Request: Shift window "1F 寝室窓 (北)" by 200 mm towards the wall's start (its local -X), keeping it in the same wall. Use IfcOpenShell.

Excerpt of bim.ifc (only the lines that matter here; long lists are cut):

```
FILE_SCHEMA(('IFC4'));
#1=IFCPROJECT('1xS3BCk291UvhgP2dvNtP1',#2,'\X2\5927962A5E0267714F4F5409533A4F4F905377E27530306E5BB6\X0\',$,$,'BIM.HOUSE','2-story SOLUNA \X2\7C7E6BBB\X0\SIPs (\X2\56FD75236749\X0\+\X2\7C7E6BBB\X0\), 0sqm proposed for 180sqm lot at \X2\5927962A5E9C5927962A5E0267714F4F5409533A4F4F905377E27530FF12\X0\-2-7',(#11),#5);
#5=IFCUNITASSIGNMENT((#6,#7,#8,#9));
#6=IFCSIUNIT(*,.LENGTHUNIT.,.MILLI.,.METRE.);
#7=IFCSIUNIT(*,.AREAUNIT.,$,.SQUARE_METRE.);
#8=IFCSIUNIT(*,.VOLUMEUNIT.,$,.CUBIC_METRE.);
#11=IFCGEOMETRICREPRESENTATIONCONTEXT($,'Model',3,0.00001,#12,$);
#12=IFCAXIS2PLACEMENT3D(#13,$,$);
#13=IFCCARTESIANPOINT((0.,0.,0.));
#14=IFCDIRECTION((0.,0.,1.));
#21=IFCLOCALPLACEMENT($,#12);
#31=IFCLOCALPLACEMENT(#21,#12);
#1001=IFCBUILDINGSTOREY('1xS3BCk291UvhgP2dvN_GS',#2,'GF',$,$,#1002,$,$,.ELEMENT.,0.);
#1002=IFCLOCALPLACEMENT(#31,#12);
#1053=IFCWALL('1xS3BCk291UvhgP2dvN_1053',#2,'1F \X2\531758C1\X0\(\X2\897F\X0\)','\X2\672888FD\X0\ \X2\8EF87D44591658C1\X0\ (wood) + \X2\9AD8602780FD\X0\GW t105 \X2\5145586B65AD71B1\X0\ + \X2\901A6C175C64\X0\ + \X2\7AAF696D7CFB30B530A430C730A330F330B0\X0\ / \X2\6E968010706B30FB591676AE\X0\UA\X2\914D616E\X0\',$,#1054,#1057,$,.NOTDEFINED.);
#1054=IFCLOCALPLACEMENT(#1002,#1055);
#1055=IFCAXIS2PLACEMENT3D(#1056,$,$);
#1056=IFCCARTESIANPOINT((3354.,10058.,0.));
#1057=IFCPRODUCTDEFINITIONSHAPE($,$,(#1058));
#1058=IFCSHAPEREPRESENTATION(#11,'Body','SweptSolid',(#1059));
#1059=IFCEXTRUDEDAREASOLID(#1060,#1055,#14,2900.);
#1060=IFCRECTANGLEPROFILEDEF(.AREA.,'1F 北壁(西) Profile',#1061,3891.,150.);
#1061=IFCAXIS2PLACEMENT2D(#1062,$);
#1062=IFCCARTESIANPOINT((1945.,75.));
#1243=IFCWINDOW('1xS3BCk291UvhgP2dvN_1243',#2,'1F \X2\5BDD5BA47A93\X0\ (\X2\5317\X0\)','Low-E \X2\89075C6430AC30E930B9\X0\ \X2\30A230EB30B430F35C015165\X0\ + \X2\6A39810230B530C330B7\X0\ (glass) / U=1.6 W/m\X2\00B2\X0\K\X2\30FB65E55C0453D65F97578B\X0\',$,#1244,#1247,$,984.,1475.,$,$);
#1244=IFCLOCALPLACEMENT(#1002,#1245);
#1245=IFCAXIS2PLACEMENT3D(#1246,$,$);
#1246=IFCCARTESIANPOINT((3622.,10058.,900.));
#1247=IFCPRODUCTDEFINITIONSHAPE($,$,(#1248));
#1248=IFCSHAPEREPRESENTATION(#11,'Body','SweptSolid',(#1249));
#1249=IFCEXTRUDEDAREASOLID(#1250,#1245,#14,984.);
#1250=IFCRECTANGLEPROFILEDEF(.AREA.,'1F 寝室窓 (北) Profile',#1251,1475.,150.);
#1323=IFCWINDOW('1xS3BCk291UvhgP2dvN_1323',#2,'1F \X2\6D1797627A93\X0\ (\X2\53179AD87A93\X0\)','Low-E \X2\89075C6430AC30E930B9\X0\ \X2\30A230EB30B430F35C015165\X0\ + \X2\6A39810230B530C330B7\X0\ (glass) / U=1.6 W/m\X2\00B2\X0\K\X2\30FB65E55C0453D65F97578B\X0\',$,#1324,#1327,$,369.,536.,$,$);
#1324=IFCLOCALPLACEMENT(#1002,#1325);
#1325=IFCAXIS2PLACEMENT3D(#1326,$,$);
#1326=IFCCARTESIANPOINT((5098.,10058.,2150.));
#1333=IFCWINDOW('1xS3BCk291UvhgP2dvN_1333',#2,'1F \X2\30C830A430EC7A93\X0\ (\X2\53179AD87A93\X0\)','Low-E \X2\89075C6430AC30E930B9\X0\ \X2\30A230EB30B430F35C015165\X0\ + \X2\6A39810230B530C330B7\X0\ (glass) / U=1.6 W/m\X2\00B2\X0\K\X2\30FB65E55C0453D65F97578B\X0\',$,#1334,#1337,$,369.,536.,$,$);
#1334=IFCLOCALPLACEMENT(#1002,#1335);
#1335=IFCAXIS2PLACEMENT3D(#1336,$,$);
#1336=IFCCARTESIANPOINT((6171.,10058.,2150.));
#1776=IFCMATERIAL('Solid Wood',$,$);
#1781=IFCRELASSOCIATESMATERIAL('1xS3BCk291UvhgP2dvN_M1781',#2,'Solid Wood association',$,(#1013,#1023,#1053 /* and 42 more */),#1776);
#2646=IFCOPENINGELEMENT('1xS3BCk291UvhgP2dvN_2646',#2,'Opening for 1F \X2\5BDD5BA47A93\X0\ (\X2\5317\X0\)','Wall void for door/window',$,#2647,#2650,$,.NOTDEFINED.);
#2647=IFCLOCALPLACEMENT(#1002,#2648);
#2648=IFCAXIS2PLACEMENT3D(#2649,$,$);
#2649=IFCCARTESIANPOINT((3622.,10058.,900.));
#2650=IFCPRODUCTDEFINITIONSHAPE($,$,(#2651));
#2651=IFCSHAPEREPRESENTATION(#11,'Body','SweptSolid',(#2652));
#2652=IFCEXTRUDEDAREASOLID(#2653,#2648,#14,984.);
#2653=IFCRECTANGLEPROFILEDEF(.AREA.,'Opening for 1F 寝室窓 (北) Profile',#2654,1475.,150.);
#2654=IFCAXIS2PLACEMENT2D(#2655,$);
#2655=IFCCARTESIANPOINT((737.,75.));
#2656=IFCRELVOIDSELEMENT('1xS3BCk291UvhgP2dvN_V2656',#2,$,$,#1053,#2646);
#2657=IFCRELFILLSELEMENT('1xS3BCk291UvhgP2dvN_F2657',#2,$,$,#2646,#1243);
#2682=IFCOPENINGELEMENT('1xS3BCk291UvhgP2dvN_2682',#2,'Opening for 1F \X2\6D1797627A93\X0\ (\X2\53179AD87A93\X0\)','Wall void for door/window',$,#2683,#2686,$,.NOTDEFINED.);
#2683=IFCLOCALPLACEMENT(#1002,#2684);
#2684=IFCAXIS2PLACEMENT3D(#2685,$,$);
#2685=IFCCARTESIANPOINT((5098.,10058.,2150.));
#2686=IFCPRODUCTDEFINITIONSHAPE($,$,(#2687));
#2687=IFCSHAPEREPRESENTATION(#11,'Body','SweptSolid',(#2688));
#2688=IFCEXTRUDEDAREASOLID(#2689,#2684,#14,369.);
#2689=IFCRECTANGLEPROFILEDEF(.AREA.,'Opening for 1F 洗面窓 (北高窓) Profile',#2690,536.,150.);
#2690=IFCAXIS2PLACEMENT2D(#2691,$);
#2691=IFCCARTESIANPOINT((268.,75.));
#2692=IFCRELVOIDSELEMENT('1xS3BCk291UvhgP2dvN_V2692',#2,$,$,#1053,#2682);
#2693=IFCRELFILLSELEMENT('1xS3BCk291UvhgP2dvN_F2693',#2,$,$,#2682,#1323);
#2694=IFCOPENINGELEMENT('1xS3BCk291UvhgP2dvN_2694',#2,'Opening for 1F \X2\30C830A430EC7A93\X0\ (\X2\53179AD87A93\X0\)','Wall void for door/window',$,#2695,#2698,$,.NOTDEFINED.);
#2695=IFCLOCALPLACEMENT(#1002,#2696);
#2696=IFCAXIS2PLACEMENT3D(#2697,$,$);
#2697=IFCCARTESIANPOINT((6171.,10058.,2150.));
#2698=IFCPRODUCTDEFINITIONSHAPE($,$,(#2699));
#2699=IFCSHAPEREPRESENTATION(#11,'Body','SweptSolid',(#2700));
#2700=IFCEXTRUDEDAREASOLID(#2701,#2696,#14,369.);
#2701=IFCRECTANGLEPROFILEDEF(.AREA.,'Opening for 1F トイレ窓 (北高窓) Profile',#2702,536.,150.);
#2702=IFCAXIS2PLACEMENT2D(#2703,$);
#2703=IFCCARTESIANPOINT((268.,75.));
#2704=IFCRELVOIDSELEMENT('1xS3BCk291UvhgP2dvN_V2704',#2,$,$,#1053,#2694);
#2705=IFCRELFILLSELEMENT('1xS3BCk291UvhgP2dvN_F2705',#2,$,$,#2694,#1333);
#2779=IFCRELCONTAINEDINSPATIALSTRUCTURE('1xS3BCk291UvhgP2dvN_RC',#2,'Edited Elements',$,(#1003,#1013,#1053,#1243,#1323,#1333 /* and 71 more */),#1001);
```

```python
import ifcopenshell
import ifcopenshell.api.geometry
import ifcopenshell.util.placement
import ifcopenshell.util.unit

model = ifcopenshell.open("bim.ifc")
unit_scale = ifcopenshell.util.unit.calculate_unit_scale(model)

window = model.by_id(1243)
opening = window.FillsVoids[0].RelatingOpeningElement
wall = opening.VoidsElements[0].RelatingBuildingElement

wall_matrix = ifcopenshell.util.placement.get_local_placement(wall.ObjectPlacement)
shift = wall_matrix[:3, 0] * -0.2 / unit_scale
before = ifcopenshell.util.placement.get_local_placement(window.ObjectPlacement)[:3, 3].copy()

# The window is not placed relative to its opening, so move both.
for product in (opening, window):
    matrix = ifcopenshell.util.placement.get_local_placement(product.ObjectPlacement)
    matrix[:3, 3] += shift
    ifcopenshell.api.geometry.edit_object_placement(model, product=product, matrix=matrix, is_si=False)

after = ifcopenshell.util.placement.get_local_placement(window.ObjectPlacement)[:3, 3]
print("window moved by", (after - before).round(3) + 0.0)

model.write("bim_v2.ifc")
```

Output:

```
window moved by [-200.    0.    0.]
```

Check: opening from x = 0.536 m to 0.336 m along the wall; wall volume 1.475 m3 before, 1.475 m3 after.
